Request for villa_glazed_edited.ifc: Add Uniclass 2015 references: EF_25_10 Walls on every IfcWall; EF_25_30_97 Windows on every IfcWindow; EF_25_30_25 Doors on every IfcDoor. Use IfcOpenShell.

First a look at what the model holds.

```python
import ifcopenshell

model = ifcopenshell.open("villa_glazed_edited.ifc")
print(model.schema)
print("classifications:", [c.Name for c in model.by_type("IfcClassification")])
for ifc_class in ("IfcDoor", "IfcRoof", "IfcStair", "IfcWall", "IfcWindow"):
    print(ifc_class, len(model.by_type(ifc_class)))
```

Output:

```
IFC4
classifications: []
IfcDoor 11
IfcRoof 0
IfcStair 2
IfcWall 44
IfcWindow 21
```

```python
import ifcopenshell
import ifcopenshell.api.classification

model = ifcopenshell.open("villa_glazed_edited.ifc")

system = ifcopenshell.api.classification.add_classification(model, classification="Uniclass 2015")

codes = {
    "IfcWall": ("EF_25_10", "Walls"),
    "IfcWindow": ("EF_25_30_97", "Windows"),
    "IfcDoor": ("EF_25_30_25", "Doors"),
}
for ifc_class, (code, name) in codes.items():
    products = model.by_type(ifc_class)
    ifcopenshell.api.classification.add_reference(
        model, products=products, classification=system, identification=code, name=name
    )
    print(code, len(products))

model.write("villa_glazed_edited_v2.ifc")
```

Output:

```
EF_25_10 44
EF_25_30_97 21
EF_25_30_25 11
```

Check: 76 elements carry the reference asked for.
